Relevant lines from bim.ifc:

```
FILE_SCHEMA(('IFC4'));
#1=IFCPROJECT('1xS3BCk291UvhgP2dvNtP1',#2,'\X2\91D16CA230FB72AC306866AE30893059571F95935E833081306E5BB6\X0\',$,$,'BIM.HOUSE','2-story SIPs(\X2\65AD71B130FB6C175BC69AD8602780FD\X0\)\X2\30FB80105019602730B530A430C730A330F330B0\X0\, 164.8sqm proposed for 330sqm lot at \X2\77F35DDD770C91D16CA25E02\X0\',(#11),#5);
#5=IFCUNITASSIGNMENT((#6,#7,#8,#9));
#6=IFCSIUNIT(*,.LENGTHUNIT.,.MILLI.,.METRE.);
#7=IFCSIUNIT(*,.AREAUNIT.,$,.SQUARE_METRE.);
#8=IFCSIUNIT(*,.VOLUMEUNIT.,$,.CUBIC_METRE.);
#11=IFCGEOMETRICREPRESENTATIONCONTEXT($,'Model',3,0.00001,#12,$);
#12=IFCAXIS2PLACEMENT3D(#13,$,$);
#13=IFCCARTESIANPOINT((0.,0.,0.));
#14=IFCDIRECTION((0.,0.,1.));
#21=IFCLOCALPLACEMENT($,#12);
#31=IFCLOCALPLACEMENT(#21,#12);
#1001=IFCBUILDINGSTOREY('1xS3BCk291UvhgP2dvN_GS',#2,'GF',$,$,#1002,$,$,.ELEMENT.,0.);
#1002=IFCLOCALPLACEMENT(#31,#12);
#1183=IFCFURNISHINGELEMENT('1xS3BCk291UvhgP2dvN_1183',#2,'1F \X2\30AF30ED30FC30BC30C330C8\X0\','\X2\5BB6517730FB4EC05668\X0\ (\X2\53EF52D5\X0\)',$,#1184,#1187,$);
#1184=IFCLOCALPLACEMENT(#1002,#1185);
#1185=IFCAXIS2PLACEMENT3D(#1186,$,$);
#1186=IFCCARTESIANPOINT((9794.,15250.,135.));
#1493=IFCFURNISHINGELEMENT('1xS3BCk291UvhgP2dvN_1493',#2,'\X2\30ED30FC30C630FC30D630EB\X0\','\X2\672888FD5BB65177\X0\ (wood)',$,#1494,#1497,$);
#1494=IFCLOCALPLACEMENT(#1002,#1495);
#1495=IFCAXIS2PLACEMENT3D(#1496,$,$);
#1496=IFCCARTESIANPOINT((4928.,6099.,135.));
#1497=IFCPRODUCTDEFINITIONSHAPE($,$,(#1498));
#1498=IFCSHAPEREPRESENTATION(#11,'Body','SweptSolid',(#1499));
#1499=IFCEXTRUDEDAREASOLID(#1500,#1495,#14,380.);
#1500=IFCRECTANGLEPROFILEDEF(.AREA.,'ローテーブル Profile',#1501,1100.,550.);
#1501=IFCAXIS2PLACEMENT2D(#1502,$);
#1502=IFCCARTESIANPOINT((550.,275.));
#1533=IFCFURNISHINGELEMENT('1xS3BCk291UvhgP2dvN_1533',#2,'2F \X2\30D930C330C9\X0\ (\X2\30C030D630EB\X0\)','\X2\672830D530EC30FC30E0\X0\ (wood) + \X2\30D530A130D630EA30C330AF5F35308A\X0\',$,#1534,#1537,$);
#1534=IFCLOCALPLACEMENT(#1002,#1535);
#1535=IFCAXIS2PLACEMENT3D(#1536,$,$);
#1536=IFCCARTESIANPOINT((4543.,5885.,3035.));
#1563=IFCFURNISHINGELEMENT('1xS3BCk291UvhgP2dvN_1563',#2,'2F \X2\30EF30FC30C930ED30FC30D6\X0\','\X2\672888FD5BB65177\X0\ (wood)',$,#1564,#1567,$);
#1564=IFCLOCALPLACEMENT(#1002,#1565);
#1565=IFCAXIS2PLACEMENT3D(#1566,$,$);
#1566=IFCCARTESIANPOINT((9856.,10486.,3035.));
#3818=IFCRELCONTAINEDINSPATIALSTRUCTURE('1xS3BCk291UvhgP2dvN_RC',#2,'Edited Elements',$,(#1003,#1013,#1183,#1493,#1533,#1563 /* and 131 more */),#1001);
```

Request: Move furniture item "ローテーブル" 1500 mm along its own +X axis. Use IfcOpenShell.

```python
import ifcopenshell
import ifcopenshell.api.geometry
import ifcopenshell.util.placement

model = ifcopenshell.open("bim.ifc")

item = model.by_guid("1xS3BCk291UvhgP2dvN_1493")
matrix = ifcopenshell.util.placement.get_local_placement(item.ObjectPlacement)
matrix[:3, 3] += matrix[:3, 0] * 1500.0
ifcopenshell.api.geometry.edit_object_placement(model, product=item, matrix=matrix, is_si=False)

print(ifcopenshell.util.placement.get_local_placement(item.ObjectPlacement).round(3) + 0.0)

model.write("bim_rev.ifc")
```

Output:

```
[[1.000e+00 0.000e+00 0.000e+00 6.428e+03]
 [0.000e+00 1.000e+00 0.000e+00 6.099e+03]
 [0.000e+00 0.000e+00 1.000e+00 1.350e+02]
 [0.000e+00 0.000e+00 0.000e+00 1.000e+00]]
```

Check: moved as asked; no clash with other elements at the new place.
